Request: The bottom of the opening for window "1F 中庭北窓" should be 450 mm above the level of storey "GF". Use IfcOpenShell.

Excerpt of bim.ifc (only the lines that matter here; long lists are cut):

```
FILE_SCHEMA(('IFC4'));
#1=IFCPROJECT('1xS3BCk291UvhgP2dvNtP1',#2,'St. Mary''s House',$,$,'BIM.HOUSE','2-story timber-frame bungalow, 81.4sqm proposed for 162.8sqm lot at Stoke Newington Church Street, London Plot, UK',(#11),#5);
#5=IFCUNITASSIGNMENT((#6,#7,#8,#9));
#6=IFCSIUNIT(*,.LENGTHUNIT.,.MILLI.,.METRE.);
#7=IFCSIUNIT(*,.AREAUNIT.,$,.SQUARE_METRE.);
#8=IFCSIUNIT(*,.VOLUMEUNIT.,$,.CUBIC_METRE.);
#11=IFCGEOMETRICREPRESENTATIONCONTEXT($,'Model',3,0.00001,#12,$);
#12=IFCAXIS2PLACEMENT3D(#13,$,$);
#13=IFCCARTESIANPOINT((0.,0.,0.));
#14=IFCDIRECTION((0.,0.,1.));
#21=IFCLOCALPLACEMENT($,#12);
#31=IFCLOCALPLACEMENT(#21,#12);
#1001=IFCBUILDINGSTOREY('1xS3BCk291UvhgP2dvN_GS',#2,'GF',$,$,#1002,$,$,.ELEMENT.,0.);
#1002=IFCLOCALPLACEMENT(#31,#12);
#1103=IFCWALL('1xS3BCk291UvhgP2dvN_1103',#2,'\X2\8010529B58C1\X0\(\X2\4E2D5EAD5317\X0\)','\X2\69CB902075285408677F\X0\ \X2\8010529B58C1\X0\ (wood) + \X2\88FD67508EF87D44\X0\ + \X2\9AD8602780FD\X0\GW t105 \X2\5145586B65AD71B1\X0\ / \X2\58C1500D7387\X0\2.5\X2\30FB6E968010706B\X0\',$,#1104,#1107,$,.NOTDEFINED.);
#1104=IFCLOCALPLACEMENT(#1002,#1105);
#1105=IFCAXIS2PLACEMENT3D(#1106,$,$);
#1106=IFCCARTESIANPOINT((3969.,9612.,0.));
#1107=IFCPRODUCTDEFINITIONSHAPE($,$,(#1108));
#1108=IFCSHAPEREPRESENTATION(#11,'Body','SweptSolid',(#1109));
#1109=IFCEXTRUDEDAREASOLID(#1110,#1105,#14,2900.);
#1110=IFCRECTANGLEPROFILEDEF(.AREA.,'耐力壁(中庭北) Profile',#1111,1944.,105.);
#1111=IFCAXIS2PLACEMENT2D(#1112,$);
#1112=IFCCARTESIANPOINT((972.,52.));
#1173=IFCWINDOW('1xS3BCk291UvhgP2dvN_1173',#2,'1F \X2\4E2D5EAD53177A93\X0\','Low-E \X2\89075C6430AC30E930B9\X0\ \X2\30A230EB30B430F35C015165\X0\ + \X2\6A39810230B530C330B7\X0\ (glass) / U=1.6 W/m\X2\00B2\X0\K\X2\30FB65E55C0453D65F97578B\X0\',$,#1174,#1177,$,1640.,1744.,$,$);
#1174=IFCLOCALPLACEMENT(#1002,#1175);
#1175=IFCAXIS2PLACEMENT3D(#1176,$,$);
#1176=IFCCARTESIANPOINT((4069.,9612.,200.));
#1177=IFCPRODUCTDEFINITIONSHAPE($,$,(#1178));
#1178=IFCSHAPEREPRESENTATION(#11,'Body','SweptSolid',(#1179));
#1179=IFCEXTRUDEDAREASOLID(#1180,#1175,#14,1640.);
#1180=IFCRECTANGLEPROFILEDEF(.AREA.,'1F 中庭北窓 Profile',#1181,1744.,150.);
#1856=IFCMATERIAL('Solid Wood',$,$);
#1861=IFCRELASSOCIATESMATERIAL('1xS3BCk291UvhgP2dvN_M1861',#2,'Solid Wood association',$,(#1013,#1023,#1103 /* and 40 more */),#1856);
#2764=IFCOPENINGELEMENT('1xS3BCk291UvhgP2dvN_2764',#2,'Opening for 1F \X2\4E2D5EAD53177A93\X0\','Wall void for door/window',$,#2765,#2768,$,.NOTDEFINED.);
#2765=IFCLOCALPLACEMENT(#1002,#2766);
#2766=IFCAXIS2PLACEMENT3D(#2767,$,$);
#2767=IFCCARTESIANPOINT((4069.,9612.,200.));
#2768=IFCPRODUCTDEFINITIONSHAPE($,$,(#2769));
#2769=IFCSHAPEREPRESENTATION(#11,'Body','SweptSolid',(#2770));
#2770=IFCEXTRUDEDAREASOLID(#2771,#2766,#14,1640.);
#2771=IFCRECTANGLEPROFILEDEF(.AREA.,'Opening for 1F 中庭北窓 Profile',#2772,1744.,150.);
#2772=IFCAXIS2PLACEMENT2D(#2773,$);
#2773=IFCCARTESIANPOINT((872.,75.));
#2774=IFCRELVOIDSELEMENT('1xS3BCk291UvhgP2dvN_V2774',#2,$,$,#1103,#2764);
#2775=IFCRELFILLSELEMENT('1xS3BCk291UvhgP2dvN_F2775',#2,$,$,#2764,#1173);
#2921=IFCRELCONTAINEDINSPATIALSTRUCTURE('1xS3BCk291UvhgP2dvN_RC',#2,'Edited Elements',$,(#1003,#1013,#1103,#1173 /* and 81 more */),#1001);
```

```python
import numpy as np
import ifcopenshell
import ifcopenshell.api.geometry
import ifcopenshell.geom
import ifcopenshell.util.element
import ifcopenshell.util.placement
import ifcopenshell.util.shape
import ifcopenshell.util.unit

model = ifcopenshell.open("bim.ifc")
unit_scale = ifcopenshell.util.unit.calculate_unit_scale(model)

window = model.by_guid("1xS3BCk291UvhgP2dvN_1173")
opening = window.FillsVoids[0].RelatingOpeningElement
storey = ifcopenshell.util.element.get_container(window, ifc_class="IfcBuildingStorey")
level = ifcopenshell.util.placement.get_local_placement(storey.ObjectPlacement)[2, 3]

# The opening's origin need not be at the sill, so measure its lowest point.
shape = ifcopenshell.geom.create_shape(ifcopenshell.geom.settings(), opening)
bottom = ifcopenshell.util.shape.get_shape_bottom_elevation(shape, shape.geometry) / unit_scale
dz = level + 0.45 / unit_scale - bottom

shift = np.array([0.0, 0.0, dz])
# The window is not placed relative to its opening, so move both.
for product in (opening, window):
    matrix = ifcopenshell.util.placement.get_local_placement(product.ObjectPlacement)
    matrix[:3, 3] += shift
    ifcopenshell.api.geometry.edit_object_placement(model, product=product, matrix=matrix, is_si=False)

print(f"moved by {dz * unit_scale:+.3f} m")

model.write("bim-out.ifc")
```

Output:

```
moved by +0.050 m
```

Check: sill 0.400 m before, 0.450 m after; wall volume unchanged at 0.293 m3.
